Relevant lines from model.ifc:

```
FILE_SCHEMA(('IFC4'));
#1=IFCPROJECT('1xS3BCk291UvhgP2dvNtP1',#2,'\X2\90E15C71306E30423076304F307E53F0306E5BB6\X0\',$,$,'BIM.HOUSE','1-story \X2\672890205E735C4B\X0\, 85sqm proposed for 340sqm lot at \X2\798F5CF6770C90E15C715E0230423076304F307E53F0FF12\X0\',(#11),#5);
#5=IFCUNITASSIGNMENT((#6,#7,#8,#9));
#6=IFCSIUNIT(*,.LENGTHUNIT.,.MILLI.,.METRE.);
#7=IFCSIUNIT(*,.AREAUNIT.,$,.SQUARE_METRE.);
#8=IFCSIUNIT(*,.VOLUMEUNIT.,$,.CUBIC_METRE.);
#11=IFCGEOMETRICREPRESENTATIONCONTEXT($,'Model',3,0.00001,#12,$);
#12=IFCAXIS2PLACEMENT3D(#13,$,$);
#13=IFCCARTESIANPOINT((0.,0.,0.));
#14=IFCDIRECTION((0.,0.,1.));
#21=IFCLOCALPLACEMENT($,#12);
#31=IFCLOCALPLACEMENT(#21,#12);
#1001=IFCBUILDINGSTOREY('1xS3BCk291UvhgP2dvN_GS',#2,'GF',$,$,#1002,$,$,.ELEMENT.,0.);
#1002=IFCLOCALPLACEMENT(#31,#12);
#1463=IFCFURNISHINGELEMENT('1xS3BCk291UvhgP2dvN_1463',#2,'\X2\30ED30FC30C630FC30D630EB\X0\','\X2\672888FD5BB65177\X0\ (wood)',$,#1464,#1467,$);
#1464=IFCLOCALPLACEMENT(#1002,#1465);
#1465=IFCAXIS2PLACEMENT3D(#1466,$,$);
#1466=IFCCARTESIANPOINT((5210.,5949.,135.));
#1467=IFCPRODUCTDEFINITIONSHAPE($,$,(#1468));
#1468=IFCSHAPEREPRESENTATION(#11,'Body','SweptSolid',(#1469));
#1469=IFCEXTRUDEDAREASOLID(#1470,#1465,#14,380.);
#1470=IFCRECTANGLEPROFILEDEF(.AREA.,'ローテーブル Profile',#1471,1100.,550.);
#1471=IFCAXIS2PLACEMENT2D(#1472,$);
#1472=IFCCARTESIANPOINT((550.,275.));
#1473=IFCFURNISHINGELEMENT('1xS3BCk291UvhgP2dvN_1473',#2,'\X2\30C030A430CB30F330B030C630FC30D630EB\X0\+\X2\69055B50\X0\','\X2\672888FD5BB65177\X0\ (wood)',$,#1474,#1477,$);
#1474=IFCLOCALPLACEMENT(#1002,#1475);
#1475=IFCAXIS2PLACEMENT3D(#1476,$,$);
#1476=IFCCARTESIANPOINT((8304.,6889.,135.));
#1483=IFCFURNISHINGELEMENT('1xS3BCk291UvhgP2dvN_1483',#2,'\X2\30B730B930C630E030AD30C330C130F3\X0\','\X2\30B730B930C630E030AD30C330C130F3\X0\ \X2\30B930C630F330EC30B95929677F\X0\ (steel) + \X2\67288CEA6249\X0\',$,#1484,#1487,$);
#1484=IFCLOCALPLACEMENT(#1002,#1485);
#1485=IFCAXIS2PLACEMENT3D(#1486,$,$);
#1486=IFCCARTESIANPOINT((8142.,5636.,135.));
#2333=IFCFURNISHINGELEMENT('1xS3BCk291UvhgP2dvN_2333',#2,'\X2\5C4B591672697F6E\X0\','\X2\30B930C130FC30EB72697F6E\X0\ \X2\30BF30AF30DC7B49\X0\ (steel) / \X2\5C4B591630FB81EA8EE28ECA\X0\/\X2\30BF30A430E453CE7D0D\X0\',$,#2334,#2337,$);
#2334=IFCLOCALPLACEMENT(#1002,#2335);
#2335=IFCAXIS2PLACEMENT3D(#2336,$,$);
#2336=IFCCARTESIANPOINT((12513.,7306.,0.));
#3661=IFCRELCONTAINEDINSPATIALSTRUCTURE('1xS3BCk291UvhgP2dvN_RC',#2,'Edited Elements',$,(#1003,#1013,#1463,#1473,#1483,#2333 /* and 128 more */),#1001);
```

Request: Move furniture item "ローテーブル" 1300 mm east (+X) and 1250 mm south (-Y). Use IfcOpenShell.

```python
import ifcopenshell
import ifcopenshell.api.geometry
import ifcopenshell.util.placement

model = ifcopenshell.open("model.ifc")

item = model.by_guid("1xS3BCk291UvhgP2dvN_1463")
matrix = ifcopenshell.util.placement.get_local_placement(item.ObjectPlacement)
matrix[0, 3] += 1300.0
matrix[1, 3] -= 1250.0
ifcopenshell.api.geometry.edit_object_placement(model, product=item, matrix=matrix, is_si=False)

print(ifcopenshell.util.placement.get_local_placement(item.ObjectPlacement).round(3) + 0.0)

model.write("model_rev.ifc")
```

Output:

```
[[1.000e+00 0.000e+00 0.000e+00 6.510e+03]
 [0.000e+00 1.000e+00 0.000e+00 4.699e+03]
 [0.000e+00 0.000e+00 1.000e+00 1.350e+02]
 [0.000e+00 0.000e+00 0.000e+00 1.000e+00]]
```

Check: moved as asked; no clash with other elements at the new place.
